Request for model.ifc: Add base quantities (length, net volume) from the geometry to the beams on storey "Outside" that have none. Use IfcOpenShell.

First a look at what the model holds.

```python
import ifcopenshell
import ifcopenshell.util.element
import ifcopenshell.util.unit

model = ifcopenshell.open("model.ifc")
print(model.schema)
for unit_type in ("LENGTHUNIT", "AREAUNIT", "VOLUMEUNIT"):
    print(unit_type, ifcopenshell.util.unit.calculate_unit_scale(model, unit_type))
storey = next(s for s in model.by_type("IfcBuildingStorey") if s.Name == "Outside")
beams = [e for e in ifcopenshell.util.element.get_decomposition(storey) if e.is_a("IfcBeam")]
for e in sorted(beams, key=lambda e: e.id()):
    print(e.id(), e.is_a(), e.Name, list(ifcopenshell.util.element.get_psets(e, qtos_only=True)), sep=" | ")
```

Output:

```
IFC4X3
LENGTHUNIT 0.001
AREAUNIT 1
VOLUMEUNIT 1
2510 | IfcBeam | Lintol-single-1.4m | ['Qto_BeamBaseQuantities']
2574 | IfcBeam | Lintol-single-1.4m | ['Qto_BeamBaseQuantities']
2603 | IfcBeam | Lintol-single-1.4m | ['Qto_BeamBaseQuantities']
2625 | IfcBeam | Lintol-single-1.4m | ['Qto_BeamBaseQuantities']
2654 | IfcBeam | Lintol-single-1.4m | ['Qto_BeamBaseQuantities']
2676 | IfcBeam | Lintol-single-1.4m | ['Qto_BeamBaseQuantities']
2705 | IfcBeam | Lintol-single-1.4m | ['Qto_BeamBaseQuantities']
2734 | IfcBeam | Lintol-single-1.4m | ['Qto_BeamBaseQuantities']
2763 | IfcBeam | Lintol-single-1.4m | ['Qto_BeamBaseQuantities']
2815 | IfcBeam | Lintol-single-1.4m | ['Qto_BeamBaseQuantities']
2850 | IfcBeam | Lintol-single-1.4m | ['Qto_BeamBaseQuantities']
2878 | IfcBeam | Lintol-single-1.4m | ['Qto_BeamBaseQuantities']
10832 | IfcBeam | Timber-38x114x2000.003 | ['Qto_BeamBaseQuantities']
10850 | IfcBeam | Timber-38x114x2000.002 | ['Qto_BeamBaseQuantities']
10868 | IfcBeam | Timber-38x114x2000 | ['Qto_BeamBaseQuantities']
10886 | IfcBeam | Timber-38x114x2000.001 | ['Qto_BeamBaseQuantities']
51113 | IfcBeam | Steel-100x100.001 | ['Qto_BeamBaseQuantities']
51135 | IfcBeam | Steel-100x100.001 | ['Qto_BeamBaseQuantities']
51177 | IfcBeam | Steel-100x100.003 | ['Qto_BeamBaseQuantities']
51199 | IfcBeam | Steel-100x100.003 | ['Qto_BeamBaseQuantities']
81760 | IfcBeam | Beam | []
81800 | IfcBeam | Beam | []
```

```python
import ifcopenshell
import ifcopenshell.api.pset
import ifcopenshell.geom
import ifcopenshell.util.element
import ifcopenshell.util.shape
import ifcopenshell.util.unit

model = ifcopenshell.open("model.ifc")
unit_scale = ifcopenshell.util.unit.calculate_unit_scale(model)
volume_scale = ifcopenshell.util.unit.calculate_unit_scale(model, "VOLUMEUNIT")
settings = ifcopenshell.geom.settings()

storey = next(s for s in model.by_type("IfcBuildingStorey") if s.Name == "Outside")
beams = [e for e in ifcopenshell.util.element.get_decomposition(storey) if e.is_a("IfcBeam")]

for e in sorted(beams, key=lambda e: e.id()):
    if ifcopenshell.util.element.get_psets(e, qtos_only=True, should_inherit=False):
        continue
    # Geometry comes back in metres, in the element's own axes.
    shape = ifcopenshell.geom.create_shape(settings, e)
    values = {
        "Length": ifcopenshell.util.shape.get_max_xyz(shape.geometry) / unit_scale,
        "NetVolume": ifcopenshell.util.shape.get_volume(shape.geometry) / volume_scale,
    }
    qto = ifcopenshell.api.pset.add_qto(model, product=e, name="Qto_BeamBaseQuantities")
    ifcopenshell.api.pset.edit_qto(model, qto=qto, properties=values)
    print(e.id(), {k: round(v, 3) for k, v in values.items()})

model.write("model_v2.ifc")
```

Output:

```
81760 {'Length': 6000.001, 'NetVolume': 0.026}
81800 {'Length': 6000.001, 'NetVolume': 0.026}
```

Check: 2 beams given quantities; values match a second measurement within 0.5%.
